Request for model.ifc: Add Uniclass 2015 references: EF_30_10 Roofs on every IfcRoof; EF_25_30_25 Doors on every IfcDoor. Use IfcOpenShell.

First a look at what the model holds.

```python
import ifcopenshell

model = ifcopenshell.open("model.ifc")
print(model.schema)
print("classifications:", [c.Name for c in model.by_type("IfcClassification")])
for ifc_class in ("IfcDoor", "IfcRoof", "IfcStair", "IfcWall", "IfcWindow"):
    print(ifc_class, len(model.by_type(ifc_class)))
```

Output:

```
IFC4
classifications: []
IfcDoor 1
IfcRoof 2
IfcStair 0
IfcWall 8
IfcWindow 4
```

```python
import ifcopenshell
import ifcopenshell.api.classification

model = ifcopenshell.open("model.ifc")

system = ifcopenshell.api.classification.add_classification(model, classification="Uniclass 2015")

codes = {
    "IfcRoof": ("EF_30_10", "Roofs"),
    "IfcDoor": ("EF_25_30_25", "Doors"),
}
for ifc_class, (code, name) in codes.items():
    products = model.by_type(ifc_class)
    ifcopenshell.api.classification.add_reference(
        model, products=products, classification=system, identification=code, name=name
    )
    print(code, len(products))

model.write("model_v2.ifc")
```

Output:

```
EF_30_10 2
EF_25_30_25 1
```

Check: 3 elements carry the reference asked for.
